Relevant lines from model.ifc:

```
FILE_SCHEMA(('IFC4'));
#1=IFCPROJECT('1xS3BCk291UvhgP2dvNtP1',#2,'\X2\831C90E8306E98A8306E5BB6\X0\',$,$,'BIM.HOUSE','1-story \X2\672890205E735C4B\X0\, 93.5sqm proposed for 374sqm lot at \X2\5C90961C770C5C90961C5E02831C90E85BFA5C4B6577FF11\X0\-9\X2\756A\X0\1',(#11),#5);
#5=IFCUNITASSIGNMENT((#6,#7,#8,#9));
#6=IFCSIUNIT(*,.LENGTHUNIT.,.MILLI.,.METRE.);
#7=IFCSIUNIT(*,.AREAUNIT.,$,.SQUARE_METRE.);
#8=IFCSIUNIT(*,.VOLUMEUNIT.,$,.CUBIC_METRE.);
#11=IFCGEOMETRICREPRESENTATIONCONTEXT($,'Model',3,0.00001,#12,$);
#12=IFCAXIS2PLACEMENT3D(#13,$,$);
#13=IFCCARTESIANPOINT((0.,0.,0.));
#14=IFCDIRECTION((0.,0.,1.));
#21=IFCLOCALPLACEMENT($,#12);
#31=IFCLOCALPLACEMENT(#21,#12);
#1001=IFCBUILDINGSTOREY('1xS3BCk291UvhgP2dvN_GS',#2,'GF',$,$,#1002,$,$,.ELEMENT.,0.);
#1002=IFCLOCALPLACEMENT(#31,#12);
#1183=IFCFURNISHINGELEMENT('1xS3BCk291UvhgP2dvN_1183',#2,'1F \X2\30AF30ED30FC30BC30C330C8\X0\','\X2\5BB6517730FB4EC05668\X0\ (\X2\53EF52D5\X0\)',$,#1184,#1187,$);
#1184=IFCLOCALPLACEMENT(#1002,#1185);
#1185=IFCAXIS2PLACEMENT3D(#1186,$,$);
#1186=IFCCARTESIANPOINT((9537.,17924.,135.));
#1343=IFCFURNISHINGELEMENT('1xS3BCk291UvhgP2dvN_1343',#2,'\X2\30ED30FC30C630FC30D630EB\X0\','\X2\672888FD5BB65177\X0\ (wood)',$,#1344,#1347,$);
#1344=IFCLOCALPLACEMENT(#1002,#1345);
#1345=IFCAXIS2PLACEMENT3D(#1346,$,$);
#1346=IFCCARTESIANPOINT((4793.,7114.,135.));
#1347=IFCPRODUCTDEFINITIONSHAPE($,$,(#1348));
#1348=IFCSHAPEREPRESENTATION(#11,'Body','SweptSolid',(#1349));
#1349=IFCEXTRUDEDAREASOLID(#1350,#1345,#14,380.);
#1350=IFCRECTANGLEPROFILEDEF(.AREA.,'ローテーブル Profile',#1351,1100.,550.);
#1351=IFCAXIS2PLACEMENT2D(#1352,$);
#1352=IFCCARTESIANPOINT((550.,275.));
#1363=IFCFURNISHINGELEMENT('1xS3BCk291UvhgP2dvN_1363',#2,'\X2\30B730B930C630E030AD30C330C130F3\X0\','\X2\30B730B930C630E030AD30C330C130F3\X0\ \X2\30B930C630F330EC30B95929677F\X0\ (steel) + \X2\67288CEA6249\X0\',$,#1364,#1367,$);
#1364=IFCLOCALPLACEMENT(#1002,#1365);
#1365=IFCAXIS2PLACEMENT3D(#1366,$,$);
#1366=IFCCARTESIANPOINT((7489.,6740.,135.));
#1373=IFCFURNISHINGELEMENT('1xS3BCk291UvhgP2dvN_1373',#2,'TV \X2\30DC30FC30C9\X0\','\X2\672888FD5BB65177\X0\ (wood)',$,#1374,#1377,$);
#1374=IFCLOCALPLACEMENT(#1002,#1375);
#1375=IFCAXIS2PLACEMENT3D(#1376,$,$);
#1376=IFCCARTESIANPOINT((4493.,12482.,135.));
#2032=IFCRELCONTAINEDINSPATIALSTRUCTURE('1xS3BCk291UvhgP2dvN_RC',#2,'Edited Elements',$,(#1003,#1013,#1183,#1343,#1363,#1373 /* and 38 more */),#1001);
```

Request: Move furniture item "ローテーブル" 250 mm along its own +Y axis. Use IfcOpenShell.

```python
import ifcopenshell
import ifcopenshell.api.geometry
import ifcopenshell.util.placement
import ifcopenshell.util.unit

model = ifcopenshell.open("model.ifc")
unit_scale = ifcopenshell.util.unit.calculate_unit_scale(model)

item = model.by_id(1343)
matrix = ifcopenshell.util.placement.get_local_placement(item.ObjectPlacement)
matrix[:3, 3] += matrix[:3, 1] * 0.25 / unit_scale
ifcopenshell.api.geometry.edit_object_placement(model, product=item, matrix=matrix, is_si=False)

print(ifcopenshell.util.placement.get_local_placement(item.ObjectPlacement).round(3) + 0.0)

model.write("model_updated.ifc")
```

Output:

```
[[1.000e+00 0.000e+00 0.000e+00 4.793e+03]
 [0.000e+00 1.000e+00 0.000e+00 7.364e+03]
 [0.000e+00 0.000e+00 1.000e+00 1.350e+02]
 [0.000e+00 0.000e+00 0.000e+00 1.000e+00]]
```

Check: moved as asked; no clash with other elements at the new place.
